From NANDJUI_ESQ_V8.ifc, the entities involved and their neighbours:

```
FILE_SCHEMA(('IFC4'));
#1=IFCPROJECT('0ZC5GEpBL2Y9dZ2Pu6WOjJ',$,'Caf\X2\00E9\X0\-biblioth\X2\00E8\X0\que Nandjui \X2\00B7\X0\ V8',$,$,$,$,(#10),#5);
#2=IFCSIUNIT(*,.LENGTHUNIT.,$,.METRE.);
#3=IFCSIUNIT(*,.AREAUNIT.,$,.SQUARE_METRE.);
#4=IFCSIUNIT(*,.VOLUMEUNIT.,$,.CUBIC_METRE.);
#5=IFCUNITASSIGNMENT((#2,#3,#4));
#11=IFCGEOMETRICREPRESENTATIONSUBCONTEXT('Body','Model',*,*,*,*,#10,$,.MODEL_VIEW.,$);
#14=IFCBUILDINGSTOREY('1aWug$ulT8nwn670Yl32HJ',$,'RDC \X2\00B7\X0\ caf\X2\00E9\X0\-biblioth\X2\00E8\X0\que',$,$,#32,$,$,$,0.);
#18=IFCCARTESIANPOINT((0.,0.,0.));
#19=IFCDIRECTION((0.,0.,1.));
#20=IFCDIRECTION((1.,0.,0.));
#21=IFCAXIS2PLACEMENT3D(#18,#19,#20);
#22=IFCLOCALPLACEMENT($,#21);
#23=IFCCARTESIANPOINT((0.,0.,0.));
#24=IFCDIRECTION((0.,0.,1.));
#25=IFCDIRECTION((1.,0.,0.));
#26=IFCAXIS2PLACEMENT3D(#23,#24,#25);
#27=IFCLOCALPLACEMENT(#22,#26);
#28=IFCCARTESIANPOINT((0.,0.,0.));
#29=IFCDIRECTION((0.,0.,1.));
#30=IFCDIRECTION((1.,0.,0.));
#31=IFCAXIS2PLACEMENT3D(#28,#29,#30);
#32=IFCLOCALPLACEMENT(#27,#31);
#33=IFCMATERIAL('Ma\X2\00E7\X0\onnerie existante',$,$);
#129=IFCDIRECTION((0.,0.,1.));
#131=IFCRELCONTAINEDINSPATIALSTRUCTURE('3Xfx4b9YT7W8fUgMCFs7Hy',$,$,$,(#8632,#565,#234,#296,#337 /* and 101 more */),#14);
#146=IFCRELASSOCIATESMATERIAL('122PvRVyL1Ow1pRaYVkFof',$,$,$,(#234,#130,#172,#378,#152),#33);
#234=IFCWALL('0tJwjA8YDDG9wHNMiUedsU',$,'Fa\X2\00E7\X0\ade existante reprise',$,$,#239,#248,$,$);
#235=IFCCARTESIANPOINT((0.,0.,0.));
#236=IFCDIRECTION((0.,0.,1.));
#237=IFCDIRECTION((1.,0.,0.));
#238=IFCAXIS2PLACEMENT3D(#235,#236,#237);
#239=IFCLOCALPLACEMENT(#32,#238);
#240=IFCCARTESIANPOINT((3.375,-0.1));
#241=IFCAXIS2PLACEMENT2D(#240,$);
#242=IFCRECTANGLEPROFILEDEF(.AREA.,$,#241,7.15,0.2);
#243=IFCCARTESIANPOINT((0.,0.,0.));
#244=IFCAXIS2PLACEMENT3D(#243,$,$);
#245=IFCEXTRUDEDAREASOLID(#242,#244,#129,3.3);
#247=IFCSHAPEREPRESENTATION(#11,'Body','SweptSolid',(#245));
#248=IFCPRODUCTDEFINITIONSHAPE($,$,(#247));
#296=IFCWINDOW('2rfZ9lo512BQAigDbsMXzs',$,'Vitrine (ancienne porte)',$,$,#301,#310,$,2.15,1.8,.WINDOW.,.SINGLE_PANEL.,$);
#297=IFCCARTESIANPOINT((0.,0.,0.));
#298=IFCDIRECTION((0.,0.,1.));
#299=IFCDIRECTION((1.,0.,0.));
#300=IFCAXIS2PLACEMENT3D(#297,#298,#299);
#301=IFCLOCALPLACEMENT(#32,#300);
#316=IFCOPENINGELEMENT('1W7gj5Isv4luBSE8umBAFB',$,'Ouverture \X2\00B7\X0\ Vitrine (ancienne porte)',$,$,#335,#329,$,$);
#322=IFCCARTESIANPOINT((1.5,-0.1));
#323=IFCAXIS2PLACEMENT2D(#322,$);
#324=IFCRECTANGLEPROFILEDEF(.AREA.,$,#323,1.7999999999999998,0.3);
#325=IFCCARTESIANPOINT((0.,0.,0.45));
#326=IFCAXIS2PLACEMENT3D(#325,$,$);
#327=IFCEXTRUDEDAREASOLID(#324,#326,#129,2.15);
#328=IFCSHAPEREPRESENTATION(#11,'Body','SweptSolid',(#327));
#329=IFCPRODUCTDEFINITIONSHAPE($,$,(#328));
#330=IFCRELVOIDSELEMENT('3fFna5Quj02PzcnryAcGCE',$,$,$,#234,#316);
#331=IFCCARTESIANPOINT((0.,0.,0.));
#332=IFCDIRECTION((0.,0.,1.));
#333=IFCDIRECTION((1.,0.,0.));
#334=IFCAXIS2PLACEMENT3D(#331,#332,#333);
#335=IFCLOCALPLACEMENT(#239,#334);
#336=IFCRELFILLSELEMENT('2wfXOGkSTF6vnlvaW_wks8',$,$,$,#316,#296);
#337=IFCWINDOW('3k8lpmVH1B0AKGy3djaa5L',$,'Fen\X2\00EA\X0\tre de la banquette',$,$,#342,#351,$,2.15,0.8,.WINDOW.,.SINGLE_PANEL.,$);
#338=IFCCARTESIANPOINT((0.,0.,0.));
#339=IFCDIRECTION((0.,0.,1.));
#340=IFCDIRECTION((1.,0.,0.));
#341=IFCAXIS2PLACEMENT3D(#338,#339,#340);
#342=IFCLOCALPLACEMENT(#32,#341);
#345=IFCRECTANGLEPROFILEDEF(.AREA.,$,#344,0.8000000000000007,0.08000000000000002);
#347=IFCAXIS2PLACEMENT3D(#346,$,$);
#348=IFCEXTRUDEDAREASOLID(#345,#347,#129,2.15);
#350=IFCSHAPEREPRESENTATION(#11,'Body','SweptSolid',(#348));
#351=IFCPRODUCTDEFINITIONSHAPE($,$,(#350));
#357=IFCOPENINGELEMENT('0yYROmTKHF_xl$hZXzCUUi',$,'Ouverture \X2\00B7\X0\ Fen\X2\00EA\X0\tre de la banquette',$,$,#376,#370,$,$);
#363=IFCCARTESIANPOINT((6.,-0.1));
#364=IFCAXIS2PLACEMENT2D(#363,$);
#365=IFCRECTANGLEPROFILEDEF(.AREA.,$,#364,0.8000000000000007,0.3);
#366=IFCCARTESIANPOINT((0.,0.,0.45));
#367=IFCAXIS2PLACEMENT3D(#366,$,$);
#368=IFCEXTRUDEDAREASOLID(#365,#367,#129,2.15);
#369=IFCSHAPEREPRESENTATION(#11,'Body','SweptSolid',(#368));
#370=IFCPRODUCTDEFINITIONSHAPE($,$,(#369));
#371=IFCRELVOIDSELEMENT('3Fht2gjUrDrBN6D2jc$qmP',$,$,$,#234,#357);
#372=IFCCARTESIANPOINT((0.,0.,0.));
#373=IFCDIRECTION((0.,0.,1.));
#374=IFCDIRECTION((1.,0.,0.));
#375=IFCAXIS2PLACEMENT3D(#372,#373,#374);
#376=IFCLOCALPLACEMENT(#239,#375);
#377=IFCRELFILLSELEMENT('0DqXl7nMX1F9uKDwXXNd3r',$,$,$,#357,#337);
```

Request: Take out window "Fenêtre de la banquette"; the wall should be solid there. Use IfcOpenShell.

```python
import ifcopenshell
import ifcopenshell.api.feature
import ifcopenshell.api.root
import ifcopenshell.geom
import ifcopenshell.util.shape

model = ifcopenshell.open("NANDJUI_ESQ_V8.ifc")
settings = ifcopenshell.geom.settings()


def volume(element):
    """Net volume in cubic metres, openings subtracted."""
    shape = ifcopenshell.geom.create_shape(settings, element)
    return ifcopenshell.util.shape.get_volume(shape.geometry)


window = model.by_guid("3k8lpmVH1B0AKGy3djaa5L")
opening = window.FillsVoids[0].RelatingOpeningElement
wall = opening.VoidsElements[0].RelatingBuildingElement
before = volume(wall)

ifcopenshell.api.root.remove_product(model, product=window)
ifcopenshell.api.feature.remove_feature(model, feature=opening)

after = volume(wall)

print(f"wall volume {before:.3f} -> {after:.3f} m3")

model.write("NANDJUI_ESQ_V8-out.ifc")
```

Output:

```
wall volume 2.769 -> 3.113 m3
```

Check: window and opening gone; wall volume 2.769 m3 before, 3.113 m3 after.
